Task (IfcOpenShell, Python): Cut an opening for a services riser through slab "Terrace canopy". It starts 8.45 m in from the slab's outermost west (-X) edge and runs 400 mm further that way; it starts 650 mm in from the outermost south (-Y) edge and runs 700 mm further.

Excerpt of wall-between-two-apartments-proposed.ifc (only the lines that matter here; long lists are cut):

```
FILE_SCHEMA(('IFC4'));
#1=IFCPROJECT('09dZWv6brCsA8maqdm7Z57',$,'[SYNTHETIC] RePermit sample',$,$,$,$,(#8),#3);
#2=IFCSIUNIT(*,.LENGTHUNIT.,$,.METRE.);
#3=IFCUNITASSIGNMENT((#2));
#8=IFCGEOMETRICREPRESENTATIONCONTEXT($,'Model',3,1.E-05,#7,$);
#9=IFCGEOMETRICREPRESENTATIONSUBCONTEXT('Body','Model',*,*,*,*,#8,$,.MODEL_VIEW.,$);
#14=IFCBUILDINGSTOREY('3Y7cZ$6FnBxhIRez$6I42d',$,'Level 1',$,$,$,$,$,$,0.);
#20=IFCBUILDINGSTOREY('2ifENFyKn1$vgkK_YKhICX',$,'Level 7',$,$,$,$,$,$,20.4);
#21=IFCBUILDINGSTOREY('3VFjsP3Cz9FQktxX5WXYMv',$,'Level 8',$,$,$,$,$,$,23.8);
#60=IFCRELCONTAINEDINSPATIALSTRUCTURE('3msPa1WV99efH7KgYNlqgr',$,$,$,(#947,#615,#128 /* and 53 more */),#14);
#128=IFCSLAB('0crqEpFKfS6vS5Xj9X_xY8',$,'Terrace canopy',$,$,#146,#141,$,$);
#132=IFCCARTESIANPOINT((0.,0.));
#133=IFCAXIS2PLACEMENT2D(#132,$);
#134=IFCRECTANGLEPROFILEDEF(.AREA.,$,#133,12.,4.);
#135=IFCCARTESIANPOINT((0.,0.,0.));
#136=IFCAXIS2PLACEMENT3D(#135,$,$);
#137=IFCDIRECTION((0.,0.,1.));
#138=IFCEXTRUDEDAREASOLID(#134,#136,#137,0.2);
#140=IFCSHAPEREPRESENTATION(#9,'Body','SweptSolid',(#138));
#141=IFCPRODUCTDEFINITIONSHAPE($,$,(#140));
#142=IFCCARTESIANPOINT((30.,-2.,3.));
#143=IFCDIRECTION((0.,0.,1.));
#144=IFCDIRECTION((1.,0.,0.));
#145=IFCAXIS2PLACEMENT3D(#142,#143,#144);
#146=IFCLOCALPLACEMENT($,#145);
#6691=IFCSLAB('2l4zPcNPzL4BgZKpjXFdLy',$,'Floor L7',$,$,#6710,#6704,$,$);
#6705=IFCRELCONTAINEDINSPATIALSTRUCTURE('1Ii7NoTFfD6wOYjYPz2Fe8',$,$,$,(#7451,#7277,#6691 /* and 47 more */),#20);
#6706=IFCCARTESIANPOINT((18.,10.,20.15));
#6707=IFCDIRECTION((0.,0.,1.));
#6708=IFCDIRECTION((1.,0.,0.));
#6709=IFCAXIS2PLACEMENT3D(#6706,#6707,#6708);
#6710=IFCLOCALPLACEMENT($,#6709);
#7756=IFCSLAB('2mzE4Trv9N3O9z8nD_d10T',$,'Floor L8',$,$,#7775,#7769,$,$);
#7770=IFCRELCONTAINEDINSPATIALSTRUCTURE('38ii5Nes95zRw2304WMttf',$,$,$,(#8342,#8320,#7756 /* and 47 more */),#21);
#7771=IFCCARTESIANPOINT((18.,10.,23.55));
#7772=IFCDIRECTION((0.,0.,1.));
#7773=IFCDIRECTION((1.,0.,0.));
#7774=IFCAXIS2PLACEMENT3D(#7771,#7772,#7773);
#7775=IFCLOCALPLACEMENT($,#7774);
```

```python
import numpy as np
import ifcopenshell
import ifcopenshell.api.feature
import ifcopenshell.api.geometry
import ifcopenshell.api.root
import ifcopenshell.geom
import ifcopenshell.util.placement
import ifcopenshell.util.representation
import ifcopenshell.util.shape
import ifcopenshell.util.unit

model = ifcopenshell.open("wall-between-two-apartments-proposed.ifc")
unit_scale = ifcopenshell.util.unit.calculate_unit_scale(model)
settings = ifcopenshell.geom.settings()


def volume(element):
    """Net volume in cubic metres, openings subtracted."""
    shape = ifcopenshell.geom.create_shape(settings, element)
    return ifcopenshell.util.shape.get_volume(shape.geometry)


slab = model.by_guid("0crqEpFKfS6vS5Xj9X_xY8")
before = volume(slab)

# Extent in the slab's own axes, in metres. The edges named are its -X and -Y sides.
slab_shape = ifcopenshell.geom.create_shape(settings, slab)
vertices = ifcopenshell.util.shape.get_vertices(slab_shape.geometry)
x_min, y_min, bottom = vertices.min(axis=0)
top = vertices[:, 2].max()

opening = ifcopenshell.api.root.create_entity(model, ifc_class="IfcOpeningElement", name="Services riser opening", predefined_type="OPENING")
context = ifcopenshell.util.representation.get_context(model, "Model", "Body", "MODEL_VIEW")
width, depth = 0.4, 0.7
outline = [(0.0, 0.0), (width, 0.0), (width, depth), (0.0, depth), (0.0, 0.0)]
# Overshoot both faces by 50 mm so the cut is clean.
shape = ifcopenshell.api.geometry.add_slab_representation(
    model, context=context, depth=top - bottom + 0.1, polyline=outline
)
ifcopenshell.api.geometry.assign_representation(model, product=opening, representation=shape)

matrix = ifcopenshell.util.placement.get_local_placement(slab.ObjectPlacement)
matrix[:, 3] = matrix @ np.append(np.array([x_min + 8.45, y_min + 0.65, bottom - 0.05]) / unit_scale, 1.0)
ifcopenshell.api.geometry.edit_object_placement(model, product=opening, matrix=matrix, is_si=False)
ifcopenshell.api.feature.add_feature(model, feature=opening, element=slab)

after = volume(slab)

print(f"slab volume {before:.3f} -> {after:.3f} m3")

model.write("wall-between-two-apartments-proposed_rev.ifc")
```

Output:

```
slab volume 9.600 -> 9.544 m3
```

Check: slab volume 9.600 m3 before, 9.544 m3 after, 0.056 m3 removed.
